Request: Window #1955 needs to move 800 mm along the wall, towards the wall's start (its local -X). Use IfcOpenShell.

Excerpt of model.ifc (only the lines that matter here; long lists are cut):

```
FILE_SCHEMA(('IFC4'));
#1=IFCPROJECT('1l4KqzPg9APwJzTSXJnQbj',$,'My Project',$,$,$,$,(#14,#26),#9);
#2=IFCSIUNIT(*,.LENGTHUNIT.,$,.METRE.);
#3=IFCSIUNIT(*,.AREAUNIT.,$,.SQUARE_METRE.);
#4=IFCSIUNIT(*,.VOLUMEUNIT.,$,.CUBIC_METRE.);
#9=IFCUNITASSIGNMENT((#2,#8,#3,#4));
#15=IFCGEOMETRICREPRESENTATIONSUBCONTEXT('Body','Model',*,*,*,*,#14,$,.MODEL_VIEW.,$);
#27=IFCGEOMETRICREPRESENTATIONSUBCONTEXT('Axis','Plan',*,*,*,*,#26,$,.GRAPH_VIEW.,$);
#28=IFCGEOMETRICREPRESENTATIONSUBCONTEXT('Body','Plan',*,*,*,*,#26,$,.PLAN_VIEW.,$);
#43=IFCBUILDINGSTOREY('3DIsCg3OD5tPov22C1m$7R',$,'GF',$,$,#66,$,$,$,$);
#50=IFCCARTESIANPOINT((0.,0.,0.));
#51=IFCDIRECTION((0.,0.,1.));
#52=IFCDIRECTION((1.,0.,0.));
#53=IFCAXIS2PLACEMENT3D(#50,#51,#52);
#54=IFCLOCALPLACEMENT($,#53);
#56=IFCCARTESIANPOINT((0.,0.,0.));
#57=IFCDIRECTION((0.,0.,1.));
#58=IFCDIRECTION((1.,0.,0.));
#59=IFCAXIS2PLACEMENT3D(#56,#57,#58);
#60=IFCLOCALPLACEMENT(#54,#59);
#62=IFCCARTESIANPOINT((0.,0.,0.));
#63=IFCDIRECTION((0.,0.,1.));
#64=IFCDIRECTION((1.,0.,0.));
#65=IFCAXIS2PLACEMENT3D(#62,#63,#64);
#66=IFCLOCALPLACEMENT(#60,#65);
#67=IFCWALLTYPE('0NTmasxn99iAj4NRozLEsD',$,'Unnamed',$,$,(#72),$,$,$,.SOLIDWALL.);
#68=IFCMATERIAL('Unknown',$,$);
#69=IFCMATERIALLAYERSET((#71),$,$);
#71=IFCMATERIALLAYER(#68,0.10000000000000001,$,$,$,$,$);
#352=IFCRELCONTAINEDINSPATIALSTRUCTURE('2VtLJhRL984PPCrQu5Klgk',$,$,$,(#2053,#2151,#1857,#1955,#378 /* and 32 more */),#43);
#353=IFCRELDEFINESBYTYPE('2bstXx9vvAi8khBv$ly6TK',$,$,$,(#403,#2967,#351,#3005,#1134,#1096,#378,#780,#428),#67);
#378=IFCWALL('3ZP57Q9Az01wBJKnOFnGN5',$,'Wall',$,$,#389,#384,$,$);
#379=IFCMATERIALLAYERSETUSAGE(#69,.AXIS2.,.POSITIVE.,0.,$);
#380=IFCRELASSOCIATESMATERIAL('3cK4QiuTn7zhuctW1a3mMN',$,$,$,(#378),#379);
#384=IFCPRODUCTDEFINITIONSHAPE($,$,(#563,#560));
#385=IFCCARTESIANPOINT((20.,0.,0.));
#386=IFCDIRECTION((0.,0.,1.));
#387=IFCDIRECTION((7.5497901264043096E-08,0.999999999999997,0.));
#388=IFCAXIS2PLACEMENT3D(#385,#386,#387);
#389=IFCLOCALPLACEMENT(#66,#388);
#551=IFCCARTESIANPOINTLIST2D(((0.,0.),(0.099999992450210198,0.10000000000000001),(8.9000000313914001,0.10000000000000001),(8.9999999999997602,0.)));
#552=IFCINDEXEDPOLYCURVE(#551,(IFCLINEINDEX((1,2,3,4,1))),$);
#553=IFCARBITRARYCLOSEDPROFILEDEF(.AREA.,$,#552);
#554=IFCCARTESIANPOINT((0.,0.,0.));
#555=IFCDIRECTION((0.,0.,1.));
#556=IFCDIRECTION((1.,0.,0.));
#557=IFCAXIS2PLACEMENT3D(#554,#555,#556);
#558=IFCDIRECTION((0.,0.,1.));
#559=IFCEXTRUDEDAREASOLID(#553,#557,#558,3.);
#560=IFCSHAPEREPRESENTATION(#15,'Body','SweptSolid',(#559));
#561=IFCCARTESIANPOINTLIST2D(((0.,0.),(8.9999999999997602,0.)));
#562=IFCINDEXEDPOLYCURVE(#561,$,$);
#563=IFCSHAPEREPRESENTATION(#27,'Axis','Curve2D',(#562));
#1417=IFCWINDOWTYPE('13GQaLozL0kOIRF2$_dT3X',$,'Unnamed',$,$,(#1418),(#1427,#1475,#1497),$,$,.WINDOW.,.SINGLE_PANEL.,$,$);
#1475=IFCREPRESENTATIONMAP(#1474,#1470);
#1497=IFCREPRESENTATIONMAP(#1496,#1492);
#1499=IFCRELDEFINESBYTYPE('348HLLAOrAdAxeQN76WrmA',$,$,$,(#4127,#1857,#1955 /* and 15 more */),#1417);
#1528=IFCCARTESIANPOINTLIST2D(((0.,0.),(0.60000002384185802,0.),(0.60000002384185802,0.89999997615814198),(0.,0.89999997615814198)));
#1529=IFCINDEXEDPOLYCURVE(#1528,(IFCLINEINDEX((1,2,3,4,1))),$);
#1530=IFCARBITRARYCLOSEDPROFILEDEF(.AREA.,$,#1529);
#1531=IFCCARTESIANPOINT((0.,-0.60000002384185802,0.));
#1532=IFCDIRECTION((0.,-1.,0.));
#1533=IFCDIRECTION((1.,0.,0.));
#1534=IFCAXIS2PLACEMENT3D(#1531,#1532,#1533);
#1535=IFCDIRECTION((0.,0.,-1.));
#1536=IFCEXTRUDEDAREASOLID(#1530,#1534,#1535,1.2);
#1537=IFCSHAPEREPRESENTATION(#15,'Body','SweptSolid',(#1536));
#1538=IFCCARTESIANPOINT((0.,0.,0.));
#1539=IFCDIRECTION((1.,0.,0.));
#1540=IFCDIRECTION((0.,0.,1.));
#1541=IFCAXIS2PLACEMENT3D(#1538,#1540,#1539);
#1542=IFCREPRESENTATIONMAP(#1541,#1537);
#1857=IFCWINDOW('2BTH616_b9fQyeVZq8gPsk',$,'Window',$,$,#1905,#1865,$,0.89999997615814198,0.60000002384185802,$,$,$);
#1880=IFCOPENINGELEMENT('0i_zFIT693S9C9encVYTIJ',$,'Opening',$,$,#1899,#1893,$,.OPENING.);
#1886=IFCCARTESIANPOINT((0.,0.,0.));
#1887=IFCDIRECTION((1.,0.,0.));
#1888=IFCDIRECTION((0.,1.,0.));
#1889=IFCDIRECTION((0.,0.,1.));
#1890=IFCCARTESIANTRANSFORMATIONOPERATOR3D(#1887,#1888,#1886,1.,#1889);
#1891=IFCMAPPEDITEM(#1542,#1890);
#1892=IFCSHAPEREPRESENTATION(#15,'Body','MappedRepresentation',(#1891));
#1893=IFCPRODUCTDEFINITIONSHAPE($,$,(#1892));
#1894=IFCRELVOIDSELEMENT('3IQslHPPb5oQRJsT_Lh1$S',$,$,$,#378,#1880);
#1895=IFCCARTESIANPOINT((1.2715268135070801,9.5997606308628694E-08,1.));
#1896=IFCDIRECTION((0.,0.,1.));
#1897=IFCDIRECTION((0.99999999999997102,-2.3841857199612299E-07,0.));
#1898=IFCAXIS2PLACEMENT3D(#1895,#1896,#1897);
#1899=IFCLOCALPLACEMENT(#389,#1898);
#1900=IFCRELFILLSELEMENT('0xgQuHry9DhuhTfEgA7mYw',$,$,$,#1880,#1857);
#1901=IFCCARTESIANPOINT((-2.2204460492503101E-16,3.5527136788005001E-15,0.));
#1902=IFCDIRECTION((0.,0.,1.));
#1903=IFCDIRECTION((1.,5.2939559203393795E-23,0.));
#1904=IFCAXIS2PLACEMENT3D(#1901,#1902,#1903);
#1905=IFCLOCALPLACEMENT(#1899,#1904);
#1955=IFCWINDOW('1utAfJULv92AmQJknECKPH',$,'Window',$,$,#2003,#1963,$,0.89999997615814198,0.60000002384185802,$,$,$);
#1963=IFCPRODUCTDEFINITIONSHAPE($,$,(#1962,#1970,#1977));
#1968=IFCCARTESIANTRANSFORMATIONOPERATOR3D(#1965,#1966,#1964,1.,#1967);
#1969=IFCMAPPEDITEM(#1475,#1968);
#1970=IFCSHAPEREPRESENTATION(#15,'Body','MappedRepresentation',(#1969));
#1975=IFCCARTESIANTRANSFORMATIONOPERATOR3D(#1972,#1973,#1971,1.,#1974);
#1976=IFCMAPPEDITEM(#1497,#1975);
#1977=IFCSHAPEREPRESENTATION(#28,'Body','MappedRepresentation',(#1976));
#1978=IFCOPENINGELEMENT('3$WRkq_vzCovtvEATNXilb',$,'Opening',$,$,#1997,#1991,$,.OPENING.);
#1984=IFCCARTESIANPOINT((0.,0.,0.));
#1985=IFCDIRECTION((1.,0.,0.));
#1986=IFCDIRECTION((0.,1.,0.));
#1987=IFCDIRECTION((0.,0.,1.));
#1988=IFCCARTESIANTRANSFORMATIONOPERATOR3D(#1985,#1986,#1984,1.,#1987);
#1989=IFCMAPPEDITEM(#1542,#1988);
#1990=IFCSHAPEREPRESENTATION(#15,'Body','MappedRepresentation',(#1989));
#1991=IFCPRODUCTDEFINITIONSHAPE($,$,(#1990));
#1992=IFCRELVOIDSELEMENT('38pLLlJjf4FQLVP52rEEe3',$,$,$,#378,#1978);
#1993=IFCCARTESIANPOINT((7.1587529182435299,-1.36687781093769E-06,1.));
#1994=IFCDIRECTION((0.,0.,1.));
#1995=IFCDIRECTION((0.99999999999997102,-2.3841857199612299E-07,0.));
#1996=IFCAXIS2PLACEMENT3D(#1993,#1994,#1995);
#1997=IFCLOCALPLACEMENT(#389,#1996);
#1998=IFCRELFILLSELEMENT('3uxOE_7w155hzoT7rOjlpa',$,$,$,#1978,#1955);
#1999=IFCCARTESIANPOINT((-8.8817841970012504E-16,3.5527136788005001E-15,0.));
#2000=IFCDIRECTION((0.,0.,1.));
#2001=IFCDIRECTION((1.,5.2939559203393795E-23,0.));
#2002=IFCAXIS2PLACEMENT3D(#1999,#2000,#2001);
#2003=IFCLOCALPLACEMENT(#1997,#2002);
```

```python
import ifcopenshell
import ifcopenshell.api.geometry
import ifcopenshell.util.placement

model = ifcopenshell.open("model.ifc")

window = model.by_id(1955)
opening = window.FillsVoids[0].RelatingOpeningElement
wall = opening.VoidsElements[0].RelatingBuildingElement

wall_matrix = ifcopenshell.util.placement.get_local_placement(wall.ObjectPlacement)
shift = wall_matrix[:3, 0] * -0.8
before = ifcopenshell.util.placement.get_local_placement(window.ObjectPlacement)[:3, 3].copy()

# The window is placed relative to its opening, so it follows when the opening moves.
matrix = ifcopenshell.util.placement.get_local_placement(opening.ObjectPlacement)
matrix[:3, 3] += shift
ifcopenshell.api.geometry.edit_object_placement(
    model, product=opening, matrix=matrix, is_si=False, should_transform_children=True
)

after = ifcopenshell.util.placement.get_local_placement(window.ObjectPlacement)[:3, 3]
print("window moved by", (after - before).round(3) + 0.0)

model.write("model_edited.ifc")
```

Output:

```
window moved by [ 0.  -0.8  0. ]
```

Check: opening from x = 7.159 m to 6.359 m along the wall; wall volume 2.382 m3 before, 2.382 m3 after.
